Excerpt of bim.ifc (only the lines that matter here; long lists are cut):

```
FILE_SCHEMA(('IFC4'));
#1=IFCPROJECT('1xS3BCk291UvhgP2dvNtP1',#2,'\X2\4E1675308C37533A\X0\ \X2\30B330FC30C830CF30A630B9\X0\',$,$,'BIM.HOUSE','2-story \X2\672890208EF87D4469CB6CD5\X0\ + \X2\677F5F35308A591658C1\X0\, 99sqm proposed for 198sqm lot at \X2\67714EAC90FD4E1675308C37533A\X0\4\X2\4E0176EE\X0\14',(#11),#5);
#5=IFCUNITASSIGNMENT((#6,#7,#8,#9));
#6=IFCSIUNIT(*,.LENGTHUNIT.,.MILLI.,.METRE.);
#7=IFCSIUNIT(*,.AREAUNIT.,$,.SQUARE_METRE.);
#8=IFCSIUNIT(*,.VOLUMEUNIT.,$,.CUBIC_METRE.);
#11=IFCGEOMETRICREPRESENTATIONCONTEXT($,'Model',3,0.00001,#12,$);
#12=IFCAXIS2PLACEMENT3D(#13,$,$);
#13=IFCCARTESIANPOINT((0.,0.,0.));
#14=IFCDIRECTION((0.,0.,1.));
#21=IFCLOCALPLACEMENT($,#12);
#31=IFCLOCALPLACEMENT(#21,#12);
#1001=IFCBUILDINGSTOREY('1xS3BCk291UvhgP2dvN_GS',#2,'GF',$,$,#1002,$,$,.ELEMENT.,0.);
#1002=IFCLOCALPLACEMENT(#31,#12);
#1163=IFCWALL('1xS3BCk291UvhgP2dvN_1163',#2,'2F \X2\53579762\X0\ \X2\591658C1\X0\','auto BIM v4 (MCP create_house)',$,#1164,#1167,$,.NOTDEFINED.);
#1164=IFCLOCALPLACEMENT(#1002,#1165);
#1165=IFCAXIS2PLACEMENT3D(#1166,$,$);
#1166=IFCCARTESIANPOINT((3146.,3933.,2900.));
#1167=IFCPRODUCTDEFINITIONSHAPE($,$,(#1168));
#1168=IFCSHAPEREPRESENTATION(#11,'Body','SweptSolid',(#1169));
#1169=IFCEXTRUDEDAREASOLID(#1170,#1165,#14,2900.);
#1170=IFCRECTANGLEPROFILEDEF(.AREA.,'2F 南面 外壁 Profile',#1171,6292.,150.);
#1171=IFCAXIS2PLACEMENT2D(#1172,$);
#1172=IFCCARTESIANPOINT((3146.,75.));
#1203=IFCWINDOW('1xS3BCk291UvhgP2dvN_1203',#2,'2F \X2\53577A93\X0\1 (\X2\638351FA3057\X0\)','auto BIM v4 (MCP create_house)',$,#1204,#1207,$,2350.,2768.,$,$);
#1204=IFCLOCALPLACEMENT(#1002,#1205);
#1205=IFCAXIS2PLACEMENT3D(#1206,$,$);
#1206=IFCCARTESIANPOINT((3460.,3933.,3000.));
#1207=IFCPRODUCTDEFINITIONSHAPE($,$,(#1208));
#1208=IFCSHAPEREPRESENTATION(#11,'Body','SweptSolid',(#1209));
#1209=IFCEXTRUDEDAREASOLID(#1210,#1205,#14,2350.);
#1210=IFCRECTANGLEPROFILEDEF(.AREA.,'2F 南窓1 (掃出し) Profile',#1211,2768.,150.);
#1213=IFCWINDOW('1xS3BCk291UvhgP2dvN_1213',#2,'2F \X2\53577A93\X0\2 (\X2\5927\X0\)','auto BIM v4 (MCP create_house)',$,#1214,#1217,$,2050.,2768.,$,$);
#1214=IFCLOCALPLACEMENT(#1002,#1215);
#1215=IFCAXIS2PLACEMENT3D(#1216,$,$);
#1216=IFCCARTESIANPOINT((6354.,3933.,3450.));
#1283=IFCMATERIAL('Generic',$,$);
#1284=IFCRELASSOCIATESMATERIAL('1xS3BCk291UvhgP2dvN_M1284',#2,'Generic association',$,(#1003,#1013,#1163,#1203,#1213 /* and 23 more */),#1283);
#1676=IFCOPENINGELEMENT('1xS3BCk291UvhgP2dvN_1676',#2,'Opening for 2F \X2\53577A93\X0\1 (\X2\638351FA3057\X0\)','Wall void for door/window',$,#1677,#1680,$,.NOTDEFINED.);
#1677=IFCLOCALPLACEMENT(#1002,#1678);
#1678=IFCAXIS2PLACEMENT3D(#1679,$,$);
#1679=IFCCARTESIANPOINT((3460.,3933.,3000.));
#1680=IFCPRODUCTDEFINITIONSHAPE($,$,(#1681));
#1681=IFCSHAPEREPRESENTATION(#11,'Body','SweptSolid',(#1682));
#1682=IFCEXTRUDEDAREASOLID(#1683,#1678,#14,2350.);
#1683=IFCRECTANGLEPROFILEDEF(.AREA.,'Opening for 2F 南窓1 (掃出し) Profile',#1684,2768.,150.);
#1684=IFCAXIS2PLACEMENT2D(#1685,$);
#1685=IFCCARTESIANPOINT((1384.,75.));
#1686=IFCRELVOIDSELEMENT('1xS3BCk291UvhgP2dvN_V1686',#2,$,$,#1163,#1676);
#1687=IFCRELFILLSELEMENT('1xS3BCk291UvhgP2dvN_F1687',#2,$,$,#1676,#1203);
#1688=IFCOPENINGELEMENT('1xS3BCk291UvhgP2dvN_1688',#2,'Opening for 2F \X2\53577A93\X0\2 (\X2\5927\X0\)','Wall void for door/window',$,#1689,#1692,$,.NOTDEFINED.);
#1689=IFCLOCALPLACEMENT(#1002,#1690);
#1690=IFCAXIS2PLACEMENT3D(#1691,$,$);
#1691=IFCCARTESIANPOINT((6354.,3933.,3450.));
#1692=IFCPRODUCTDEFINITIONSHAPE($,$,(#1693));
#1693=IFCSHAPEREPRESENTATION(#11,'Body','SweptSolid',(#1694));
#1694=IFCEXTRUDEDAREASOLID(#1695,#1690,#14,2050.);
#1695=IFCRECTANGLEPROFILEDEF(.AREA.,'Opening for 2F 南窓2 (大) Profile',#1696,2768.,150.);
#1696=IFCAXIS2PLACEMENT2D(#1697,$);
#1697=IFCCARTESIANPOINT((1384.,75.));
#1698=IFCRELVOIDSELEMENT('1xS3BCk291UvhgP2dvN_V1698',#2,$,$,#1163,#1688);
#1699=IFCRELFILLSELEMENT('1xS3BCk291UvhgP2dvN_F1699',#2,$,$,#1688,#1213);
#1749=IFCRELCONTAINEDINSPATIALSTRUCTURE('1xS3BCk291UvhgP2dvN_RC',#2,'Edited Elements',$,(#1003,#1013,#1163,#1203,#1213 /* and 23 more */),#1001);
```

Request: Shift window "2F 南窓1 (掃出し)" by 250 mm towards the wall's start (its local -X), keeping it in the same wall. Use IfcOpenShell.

```python
import ifcopenshell
import ifcopenshell.api.geometry
import ifcopenshell.util.placement

model = ifcopenshell.open("bim.ifc")

window = model.by_guid("1xS3BCk291UvhgP2dvN_1203")
opening = window.FillsVoids[0].RelatingOpeningElement
wall = opening.VoidsElements[0].RelatingBuildingElement

wall_matrix = ifcopenshell.util.placement.get_local_placement(wall.ObjectPlacement)
shift = wall_matrix[:3, 0] * -250.0
before = ifcopenshell.util.placement.get_local_placement(window.ObjectPlacement)[:3, 3].copy()

# The window is not placed relative to its opening, so move both.
for product in (opening, window):
    matrix = ifcopenshell.util.placement.get_local_placement(product.ObjectPlacement)
    matrix[:3, 3] += shift
    ifcopenshell.api.geometry.edit_object_placement(model, product=product, matrix=matrix, is_si=False)

after = ifcopenshell.util.placement.get_local_placement(window.ObjectPlacement)[:3, 3]
print("window moved by", (after - before).round(3) + 0.0)

model.write("bim_v2.ifc")
```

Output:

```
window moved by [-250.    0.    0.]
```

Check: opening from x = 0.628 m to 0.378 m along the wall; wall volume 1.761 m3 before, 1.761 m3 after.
